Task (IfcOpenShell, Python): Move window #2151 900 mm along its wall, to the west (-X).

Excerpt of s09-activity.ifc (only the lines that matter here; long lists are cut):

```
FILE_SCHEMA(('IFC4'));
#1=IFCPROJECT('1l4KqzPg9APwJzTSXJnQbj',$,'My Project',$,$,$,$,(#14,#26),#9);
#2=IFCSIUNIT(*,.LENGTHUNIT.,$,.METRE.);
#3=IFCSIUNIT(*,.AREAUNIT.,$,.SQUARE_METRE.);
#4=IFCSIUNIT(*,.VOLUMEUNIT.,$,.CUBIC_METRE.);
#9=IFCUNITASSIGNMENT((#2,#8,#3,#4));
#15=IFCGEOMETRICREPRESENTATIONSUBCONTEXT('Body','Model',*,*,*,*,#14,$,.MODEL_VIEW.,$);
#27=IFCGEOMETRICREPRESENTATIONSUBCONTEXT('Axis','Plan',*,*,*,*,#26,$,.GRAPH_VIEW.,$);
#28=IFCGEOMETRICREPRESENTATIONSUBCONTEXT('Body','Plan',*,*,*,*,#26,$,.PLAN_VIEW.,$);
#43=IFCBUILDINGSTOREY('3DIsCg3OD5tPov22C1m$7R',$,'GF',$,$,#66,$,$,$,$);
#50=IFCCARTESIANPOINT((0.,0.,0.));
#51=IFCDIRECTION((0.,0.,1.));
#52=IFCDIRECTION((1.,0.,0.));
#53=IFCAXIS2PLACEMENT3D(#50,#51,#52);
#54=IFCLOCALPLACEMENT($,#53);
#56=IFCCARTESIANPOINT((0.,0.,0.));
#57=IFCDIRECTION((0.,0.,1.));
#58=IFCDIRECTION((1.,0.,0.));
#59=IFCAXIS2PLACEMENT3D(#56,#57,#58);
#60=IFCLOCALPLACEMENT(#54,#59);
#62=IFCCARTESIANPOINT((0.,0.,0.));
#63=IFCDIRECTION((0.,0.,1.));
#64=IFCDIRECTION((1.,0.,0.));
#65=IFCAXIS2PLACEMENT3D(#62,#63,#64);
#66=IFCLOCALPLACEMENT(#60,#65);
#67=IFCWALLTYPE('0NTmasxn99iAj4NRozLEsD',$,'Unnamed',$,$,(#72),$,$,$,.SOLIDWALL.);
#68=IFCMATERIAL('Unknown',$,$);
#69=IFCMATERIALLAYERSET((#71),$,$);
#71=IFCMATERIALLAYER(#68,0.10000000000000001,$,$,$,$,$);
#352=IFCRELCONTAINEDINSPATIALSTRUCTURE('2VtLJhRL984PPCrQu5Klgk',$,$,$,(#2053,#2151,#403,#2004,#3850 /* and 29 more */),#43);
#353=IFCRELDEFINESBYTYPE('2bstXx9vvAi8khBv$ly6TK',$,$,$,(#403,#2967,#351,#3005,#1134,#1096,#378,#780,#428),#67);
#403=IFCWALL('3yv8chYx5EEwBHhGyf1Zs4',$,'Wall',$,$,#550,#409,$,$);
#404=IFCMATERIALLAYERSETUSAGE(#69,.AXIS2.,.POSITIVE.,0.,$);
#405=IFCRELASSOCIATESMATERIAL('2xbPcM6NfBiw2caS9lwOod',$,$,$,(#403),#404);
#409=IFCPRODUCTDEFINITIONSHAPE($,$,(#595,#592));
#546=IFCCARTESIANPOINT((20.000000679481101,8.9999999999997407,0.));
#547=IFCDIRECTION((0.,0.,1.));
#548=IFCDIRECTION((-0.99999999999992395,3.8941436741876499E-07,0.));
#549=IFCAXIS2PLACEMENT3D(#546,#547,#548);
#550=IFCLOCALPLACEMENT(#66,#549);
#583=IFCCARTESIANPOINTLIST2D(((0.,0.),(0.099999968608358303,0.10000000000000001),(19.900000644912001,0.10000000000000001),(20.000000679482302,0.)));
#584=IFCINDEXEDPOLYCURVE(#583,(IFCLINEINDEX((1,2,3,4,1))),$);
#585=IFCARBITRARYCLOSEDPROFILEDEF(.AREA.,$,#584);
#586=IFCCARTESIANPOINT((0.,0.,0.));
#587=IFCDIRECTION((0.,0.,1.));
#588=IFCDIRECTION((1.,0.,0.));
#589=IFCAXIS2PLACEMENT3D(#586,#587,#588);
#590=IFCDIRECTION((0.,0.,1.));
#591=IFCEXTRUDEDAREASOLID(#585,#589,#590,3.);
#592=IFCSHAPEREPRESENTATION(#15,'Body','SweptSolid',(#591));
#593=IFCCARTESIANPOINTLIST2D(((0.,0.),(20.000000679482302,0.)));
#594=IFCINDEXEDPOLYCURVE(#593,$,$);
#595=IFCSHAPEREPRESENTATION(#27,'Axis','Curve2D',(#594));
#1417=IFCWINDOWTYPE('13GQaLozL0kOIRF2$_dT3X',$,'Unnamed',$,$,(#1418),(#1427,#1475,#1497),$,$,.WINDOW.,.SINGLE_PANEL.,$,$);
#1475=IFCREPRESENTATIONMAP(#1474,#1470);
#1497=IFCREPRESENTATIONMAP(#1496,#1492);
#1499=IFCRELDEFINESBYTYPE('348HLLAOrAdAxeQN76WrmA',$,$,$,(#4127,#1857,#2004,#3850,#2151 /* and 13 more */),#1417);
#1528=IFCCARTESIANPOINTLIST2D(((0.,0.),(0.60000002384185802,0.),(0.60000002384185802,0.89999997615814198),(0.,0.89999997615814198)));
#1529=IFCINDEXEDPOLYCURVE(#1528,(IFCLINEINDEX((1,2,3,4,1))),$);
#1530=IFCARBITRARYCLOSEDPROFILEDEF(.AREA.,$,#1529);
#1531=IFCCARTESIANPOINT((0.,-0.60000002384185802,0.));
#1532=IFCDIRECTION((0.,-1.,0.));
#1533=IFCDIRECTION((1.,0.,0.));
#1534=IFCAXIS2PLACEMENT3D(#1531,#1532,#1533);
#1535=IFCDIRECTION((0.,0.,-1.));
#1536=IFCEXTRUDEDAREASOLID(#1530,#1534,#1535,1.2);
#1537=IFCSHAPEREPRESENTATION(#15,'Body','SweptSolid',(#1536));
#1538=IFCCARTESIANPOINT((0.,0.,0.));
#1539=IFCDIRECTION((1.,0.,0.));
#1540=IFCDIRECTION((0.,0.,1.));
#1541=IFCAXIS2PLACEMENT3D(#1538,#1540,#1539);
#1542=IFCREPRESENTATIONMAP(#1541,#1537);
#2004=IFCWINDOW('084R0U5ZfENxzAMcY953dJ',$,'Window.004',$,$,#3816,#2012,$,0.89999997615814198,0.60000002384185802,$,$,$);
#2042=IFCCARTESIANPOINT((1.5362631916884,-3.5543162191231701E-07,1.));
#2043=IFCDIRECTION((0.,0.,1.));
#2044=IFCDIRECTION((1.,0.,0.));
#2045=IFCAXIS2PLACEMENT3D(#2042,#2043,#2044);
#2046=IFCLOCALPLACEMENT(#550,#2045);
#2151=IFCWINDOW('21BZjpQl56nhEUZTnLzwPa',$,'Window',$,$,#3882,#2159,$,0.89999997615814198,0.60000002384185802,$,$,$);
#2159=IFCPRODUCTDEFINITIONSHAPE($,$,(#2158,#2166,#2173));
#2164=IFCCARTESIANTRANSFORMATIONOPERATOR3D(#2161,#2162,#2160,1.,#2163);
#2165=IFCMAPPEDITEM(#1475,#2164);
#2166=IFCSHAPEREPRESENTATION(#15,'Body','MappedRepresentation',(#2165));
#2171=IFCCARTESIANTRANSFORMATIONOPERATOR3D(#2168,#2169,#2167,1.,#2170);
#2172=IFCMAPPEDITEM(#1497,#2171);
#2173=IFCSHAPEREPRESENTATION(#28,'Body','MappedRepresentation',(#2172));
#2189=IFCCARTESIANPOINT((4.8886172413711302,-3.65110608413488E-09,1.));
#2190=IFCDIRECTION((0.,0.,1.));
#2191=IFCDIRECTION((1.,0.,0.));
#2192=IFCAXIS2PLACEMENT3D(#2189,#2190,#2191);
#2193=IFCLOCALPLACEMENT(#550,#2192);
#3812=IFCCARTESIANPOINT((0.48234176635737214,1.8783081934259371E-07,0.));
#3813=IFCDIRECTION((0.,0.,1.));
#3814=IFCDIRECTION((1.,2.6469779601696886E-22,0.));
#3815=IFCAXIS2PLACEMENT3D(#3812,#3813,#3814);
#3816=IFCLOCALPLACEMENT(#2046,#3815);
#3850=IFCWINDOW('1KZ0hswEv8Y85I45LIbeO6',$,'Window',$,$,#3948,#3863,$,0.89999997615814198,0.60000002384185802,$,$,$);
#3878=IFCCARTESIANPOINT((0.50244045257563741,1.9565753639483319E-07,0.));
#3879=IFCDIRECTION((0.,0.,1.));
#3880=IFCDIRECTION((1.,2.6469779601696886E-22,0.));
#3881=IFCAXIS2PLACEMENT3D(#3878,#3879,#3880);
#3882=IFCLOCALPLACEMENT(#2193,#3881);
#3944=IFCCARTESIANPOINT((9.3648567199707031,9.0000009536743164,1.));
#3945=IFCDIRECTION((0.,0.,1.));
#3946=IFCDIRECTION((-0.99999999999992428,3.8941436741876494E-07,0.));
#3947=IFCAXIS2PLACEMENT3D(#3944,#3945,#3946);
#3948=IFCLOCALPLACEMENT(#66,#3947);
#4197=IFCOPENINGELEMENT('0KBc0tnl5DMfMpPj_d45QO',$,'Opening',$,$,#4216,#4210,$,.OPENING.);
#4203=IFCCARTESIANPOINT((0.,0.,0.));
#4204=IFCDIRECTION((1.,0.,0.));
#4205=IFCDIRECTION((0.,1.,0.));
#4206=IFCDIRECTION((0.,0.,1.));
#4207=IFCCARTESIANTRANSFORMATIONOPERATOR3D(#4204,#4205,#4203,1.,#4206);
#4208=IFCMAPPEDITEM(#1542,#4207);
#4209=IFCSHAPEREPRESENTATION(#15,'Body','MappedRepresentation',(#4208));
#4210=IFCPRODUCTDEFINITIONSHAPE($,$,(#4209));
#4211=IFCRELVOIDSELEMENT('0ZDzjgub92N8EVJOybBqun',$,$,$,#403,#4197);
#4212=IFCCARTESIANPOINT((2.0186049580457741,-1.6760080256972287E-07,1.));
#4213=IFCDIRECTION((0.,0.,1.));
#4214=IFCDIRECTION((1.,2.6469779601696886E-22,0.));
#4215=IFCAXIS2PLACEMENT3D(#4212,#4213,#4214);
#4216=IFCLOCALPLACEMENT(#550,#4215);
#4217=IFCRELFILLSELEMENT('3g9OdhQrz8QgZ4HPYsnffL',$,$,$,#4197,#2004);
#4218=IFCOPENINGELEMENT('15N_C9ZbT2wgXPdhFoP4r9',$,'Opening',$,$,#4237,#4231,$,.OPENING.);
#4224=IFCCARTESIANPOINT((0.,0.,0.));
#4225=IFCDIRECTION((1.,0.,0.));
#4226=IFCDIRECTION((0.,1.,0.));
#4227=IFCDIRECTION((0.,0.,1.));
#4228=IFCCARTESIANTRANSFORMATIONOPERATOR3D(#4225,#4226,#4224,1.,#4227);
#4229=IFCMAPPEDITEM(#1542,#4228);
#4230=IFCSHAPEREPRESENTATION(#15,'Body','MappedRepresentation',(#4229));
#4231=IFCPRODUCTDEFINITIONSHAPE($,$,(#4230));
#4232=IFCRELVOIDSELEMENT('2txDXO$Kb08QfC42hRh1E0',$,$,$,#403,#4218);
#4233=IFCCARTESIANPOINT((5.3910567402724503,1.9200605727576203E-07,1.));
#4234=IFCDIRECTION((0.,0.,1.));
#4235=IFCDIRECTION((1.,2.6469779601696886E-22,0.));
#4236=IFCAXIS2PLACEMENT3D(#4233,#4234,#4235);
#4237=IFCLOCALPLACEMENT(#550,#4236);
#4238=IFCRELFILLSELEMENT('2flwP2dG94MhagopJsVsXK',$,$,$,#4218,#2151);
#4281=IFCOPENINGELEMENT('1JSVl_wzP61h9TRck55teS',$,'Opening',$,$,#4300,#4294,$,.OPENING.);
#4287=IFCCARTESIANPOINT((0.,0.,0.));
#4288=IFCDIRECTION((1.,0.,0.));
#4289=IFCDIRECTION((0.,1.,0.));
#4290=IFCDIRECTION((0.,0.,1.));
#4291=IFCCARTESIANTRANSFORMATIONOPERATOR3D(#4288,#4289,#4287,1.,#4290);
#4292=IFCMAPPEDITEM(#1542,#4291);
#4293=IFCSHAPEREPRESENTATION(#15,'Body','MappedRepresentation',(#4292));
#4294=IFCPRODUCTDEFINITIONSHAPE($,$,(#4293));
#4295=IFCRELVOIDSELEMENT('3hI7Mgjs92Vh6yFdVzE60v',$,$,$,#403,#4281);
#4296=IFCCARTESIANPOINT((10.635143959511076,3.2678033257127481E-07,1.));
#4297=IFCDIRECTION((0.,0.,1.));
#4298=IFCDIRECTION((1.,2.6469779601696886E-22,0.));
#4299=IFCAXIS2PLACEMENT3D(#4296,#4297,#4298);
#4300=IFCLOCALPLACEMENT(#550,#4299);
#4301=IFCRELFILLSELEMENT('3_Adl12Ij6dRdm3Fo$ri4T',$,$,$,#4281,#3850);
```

```python
import ifcopenshell
import ifcopenshell.api.geometry
import ifcopenshell.util.placement
import ifcopenshell.util.unit

model = ifcopenshell.open("s09-activity.ifc")
unit_scale = ifcopenshell.util.unit.calculate_unit_scale(model)

window = model.by_guid("21BZjpQl56nhEUZTnLzwPa")
opening = window.FillsVoids[0].RelatingOpeningElement
wall = opening.VoidsElements[0].RelatingBuildingElement

wall_matrix = ifcopenshell.util.placement.get_local_placement(wall.ObjectPlacement)
shift = wall_matrix[:3, 0] * 0.9 / unit_scale
before = ifcopenshell.util.placement.get_local_placement(window.ObjectPlacement)[:3, 3].copy()

# The window is not placed relative to its opening, so move both.
for product in (opening, window):
    matrix = ifcopenshell.util.placement.get_local_placement(product.ObjectPlacement)
    matrix[:3, 3] += shift
    ifcopenshell.api.geometry.edit_object_placement(model, product=product, matrix=matrix, is_si=False)

after = ifcopenshell.util.placement.get_local_placement(window.ObjectPlacement)[:3, 3]
print("window moved by", (after - before).round(3) + 0.0)

model.write("s09-activity_updated.ifc")
```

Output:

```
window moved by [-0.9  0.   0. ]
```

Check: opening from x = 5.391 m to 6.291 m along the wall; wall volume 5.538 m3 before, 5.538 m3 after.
